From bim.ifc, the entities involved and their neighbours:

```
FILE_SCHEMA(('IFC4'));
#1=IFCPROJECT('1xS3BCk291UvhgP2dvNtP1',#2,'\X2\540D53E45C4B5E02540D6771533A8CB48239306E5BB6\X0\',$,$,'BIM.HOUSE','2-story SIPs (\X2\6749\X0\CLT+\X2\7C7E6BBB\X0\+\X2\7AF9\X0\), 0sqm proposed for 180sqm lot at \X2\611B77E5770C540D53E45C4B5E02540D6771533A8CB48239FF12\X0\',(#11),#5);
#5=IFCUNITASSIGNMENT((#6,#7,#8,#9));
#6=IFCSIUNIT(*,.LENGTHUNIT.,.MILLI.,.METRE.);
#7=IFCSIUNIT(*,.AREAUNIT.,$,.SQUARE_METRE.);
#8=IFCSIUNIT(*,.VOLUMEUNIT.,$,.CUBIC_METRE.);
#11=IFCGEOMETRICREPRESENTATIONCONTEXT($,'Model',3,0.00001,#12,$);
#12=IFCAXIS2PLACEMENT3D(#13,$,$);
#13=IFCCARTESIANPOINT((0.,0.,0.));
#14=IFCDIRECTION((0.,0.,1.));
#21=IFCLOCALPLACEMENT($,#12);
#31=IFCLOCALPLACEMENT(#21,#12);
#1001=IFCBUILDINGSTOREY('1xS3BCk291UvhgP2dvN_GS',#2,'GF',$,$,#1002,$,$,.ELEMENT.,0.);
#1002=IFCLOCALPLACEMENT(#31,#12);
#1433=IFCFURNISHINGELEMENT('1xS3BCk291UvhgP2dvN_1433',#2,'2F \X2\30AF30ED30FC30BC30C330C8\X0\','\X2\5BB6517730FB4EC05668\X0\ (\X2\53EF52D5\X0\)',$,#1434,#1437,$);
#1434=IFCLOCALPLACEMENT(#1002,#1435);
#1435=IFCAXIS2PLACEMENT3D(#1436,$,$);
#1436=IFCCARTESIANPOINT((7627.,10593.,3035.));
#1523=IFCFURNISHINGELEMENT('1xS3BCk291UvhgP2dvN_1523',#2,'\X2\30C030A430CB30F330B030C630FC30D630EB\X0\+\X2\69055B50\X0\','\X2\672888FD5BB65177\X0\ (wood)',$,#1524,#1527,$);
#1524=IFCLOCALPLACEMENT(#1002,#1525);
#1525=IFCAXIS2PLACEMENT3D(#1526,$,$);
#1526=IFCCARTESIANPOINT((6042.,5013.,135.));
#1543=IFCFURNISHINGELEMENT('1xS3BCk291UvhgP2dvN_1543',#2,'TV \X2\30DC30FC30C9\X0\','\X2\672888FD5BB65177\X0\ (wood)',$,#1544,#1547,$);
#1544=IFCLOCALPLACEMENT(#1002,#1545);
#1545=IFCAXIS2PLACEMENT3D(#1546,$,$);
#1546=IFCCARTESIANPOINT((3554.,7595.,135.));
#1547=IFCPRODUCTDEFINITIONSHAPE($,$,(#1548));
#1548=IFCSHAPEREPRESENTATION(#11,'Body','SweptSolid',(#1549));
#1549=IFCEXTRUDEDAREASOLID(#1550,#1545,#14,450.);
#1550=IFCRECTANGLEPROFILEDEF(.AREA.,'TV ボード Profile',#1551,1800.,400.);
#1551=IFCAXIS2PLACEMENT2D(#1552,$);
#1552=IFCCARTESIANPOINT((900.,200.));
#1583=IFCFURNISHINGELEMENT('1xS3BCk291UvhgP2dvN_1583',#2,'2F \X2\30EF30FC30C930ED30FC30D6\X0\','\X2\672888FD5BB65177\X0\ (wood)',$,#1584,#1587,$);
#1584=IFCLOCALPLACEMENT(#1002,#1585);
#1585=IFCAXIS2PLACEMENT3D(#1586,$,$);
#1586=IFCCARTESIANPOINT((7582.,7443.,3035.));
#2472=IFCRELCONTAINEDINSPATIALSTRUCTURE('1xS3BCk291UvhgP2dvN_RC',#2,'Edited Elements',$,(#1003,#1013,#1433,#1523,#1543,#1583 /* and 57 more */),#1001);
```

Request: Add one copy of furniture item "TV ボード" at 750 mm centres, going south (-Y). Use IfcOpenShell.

```python
import numpy as np
import ifcopenshell
import ifcopenshell.api.geometry
import ifcopenshell.api.root
import ifcopenshell.util.element
import ifcopenshell.util.placement
import ifcopenshell.util.unit

model = ifcopenshell.open("bim.ifc")
unit_scale = ifcopenshell.util.unit.calculate_unit_scale(model)


def reuse_history(source, copy):
    """copy_class also copies each property set's owner history, people and application; keep the originals."""
    for rel in copy.IsDefinedBy:
        if rel.is_a("IfcRelDefinesByProperties") and (history := rel.RelatingPropertyDefinition.OwnerHistory):
            rel.RelatingPropertyDefinition.OwnerHistory = source.OwnerHistory
            ifcopenshell.util.element.remove_deep2(model, history)


source = model.by_guid("1xS3BCk291UvhgP2dvN_1543")
base = ifcopenshell.util.placement.get_local_placement(source.ObjectPlacement)
step = np.array([0.0, -1.0, 0.0]) * 0.75 / unit_scale

for i in range(1, 2):
    copy = ifcopenshell.api.root.copy_class(model, product=source)
    copy.Representation = ifcopenshell.util.element.copy_deep(
        model, source.Representation, exclude=["IfcGeometricRepresentationContext", "IfcRepresentationMap"]
    )
    reuse_history(source, copy)
    matrix = base.copy()
    matrix[:3, 3] += i * step
    print("added at", matrix[:3, 3].round(3) + 0.0)
    ifcopenshell.api.geometry.edit_object_placement(model, product=copy, matrix=matrix, is_si=False)

model.write("bim_rev.ifc")
```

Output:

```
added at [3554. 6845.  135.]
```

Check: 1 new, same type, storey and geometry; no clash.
